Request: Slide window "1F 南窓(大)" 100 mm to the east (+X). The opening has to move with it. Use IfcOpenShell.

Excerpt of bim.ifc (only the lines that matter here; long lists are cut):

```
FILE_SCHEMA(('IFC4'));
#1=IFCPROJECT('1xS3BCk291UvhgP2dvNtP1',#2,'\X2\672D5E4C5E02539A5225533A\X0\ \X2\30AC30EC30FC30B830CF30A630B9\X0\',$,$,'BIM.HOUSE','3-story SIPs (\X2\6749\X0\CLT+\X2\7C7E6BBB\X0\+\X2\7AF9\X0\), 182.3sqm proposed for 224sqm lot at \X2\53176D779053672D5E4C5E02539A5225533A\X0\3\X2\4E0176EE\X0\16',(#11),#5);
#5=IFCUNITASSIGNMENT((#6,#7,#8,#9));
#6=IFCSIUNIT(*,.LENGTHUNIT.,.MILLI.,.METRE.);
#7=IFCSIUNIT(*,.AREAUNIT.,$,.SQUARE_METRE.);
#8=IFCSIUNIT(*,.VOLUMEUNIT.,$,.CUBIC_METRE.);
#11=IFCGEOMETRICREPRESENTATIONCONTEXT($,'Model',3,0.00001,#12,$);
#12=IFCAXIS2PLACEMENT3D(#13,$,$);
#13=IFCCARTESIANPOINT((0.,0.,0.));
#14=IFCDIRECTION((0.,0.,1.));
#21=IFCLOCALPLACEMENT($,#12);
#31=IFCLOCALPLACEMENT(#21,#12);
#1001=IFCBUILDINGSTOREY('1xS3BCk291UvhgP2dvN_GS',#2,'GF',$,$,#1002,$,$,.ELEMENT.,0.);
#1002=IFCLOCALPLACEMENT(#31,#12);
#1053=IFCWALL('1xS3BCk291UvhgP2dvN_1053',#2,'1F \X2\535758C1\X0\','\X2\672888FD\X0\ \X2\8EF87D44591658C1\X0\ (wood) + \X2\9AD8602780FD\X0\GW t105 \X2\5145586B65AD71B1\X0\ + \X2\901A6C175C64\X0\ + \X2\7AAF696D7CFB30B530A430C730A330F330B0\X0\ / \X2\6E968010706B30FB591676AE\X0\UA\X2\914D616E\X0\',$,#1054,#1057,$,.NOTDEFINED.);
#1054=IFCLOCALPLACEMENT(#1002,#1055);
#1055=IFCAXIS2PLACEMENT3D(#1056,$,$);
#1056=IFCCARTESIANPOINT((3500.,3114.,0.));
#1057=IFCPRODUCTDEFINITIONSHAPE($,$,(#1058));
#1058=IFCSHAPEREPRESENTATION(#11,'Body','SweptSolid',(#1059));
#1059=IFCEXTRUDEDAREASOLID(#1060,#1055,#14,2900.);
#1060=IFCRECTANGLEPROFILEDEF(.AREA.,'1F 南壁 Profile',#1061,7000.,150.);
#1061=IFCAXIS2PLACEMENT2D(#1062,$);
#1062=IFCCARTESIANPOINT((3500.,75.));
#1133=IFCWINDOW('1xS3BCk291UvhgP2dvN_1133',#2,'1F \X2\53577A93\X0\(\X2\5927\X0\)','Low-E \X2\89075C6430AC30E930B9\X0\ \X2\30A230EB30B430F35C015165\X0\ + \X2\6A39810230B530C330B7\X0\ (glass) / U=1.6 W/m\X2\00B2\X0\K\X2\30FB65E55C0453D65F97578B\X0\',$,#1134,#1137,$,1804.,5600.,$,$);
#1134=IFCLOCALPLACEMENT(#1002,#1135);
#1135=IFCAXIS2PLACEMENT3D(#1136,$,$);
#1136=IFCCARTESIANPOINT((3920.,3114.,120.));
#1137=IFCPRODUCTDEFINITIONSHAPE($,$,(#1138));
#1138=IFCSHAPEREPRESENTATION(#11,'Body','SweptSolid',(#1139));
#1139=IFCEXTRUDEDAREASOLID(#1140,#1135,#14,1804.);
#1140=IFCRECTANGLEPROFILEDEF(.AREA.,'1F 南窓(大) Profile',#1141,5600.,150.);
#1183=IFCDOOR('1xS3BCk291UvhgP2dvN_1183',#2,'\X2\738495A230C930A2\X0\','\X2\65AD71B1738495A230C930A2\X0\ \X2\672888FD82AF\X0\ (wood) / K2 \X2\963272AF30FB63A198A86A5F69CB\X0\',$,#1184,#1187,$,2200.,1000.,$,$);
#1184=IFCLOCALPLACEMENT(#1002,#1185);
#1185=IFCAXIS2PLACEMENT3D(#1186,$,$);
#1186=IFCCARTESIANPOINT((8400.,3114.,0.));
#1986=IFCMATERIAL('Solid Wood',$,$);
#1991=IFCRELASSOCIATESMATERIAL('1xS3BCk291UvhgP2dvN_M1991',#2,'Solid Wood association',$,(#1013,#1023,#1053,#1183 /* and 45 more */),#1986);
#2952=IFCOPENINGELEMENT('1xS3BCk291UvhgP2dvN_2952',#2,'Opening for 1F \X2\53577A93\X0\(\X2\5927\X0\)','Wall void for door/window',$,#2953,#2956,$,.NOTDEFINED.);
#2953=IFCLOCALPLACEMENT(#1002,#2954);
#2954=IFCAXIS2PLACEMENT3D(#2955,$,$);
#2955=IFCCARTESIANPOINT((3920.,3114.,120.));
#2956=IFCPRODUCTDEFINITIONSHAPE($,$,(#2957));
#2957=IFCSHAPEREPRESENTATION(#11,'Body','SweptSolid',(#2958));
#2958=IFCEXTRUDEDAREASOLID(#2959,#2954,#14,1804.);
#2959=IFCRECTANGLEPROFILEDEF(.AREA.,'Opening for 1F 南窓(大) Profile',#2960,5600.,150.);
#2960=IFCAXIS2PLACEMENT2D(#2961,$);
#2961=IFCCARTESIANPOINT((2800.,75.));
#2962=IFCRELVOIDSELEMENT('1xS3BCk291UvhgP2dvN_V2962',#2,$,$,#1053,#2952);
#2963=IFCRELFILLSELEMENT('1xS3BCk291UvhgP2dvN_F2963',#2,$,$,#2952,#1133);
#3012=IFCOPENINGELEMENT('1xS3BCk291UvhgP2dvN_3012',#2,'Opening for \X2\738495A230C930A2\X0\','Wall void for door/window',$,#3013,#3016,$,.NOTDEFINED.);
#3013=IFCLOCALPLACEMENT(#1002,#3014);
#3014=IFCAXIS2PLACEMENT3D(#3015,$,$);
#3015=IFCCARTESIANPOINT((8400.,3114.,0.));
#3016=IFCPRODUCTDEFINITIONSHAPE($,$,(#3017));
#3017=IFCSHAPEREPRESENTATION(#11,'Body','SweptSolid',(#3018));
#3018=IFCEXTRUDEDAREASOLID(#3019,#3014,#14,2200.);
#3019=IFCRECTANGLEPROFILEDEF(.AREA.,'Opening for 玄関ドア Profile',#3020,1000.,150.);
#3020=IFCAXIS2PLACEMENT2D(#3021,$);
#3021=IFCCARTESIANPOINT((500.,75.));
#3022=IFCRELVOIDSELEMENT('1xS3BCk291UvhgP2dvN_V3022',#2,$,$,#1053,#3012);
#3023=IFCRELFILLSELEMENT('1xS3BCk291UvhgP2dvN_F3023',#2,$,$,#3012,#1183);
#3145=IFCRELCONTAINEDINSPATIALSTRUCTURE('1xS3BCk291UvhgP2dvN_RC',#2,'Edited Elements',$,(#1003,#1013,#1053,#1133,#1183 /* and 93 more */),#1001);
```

```python
import ifcopenshell
import ifcopenshell.api.geometry
import ifcopenshell.util.placement

model = ifcopenshell.open("bim.ifc")

window = model.by_guid("1xS3BCk291UvhgP2dvN_1133")
opening = window.FillsVoids[0].RelatingOpeningElement
wall = opening.VoidsElements[0].RelatingBuildingElement

wall_matrix = ifcopenshell.util.placement.get_local_placement(wall.ObjectPlacement)
shift = wall_matrix[:3, 0] * 100.0
before = ifcopenshell.util.placement.get_local_placement(window.ObjectPlacement)[:3, 3].copy()

# The window is not placed relative to its opening, so move both.
for product in (opening, window):
    matrix = ifcopenshell.util.placement.get_local_placement(product.ObjectPlacement)
    matrix[:3, 3] += shift
    ifcopenshell.api.geometry.edit_object_placement(model, product=product, matrix=matrix, is_si=False)

after = ifcopenshell.util.placement.get_local_placement(window.ObjectPlacement)[:3, 3]
print("window moved by", (after - before).round(3) + 0.0)

model.write("bim_updated.ifc")
```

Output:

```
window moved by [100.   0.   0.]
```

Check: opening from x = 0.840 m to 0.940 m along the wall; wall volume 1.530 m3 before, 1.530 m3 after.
